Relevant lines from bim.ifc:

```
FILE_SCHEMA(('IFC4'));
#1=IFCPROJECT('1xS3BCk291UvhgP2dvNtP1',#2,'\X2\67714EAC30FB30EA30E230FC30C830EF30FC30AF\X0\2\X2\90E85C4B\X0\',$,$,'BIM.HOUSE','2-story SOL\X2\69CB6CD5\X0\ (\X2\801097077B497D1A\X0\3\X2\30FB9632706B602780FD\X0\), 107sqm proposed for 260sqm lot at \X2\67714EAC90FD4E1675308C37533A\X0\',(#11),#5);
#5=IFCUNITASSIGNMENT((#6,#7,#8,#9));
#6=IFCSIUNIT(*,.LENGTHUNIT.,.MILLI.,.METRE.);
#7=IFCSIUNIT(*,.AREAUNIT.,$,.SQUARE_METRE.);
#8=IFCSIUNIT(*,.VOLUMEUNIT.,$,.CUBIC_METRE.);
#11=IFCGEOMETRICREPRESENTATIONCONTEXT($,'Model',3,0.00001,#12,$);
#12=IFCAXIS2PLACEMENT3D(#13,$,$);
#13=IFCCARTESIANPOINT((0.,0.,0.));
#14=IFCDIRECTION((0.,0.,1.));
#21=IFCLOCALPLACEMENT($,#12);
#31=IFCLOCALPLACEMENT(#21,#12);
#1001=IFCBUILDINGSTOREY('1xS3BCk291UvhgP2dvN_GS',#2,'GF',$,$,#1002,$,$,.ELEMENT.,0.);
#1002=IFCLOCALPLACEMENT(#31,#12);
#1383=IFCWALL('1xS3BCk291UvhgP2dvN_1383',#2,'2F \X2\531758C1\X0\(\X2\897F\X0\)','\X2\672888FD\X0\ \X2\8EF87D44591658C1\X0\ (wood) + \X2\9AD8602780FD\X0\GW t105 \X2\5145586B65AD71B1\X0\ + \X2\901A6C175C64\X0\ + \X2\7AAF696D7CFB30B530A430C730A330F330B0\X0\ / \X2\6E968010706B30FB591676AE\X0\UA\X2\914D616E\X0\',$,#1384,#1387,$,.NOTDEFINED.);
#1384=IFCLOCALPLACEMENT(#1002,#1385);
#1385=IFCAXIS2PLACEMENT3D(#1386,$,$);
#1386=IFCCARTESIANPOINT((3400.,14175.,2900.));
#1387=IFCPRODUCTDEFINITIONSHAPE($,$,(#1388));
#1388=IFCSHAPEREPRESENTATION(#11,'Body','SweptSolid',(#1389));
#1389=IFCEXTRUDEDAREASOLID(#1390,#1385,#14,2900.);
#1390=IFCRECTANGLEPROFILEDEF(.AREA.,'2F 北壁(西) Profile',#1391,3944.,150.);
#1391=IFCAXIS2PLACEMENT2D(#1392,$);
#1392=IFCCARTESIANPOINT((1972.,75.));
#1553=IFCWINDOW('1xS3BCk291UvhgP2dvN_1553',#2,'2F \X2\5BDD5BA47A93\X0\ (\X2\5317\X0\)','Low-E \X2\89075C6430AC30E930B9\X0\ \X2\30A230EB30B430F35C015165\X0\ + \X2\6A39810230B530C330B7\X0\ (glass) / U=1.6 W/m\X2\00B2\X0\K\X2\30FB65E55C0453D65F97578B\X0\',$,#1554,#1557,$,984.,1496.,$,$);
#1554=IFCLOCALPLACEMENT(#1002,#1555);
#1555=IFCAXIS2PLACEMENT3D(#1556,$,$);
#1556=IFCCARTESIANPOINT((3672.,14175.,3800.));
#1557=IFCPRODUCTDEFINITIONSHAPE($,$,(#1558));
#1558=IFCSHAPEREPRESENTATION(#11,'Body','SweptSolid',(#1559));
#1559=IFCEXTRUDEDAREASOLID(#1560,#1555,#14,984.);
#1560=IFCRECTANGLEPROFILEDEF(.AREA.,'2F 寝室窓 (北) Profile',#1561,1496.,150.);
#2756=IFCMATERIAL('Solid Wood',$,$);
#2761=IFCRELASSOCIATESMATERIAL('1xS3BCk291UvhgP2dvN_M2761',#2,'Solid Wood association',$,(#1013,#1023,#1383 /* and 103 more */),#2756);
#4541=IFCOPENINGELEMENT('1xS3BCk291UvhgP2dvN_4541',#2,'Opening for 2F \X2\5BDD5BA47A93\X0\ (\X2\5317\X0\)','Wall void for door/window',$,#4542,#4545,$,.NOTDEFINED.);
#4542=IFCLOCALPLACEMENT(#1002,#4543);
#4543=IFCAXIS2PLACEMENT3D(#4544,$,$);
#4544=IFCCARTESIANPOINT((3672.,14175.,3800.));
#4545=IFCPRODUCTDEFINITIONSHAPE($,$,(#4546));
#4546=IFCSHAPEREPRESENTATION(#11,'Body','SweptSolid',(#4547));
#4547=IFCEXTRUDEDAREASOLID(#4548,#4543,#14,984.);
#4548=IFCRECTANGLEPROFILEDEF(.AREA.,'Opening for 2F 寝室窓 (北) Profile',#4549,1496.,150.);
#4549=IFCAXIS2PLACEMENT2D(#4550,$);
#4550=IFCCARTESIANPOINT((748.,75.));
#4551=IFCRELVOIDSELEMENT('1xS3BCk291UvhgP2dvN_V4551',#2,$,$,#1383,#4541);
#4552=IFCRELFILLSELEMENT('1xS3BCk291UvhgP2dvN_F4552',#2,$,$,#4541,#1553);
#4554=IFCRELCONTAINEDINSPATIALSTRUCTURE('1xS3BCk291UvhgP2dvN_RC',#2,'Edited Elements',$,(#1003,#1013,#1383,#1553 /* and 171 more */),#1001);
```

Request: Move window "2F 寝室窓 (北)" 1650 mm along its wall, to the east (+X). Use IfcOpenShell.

```python
import ifcopenshell
import ifcopenshell.api.geometry
import ifcopenshell.util.placement
import ifcopenshell.util.unit

model = ifcopenshell.open("bim.ifc")
unit_scale = ifcopenshell.util.unit.calculate_unit_scale(model)

window = model.by_id(1553)
opening = window.FillsVoids[0].RelatingOpeningElement
wall = opening.VoidsElements[0].RelatingBuildingElement

wall_matrix = ifcopenshell.util.placement.get_local_placement(wall.ObjectPlacement)
shift = wall_matrix[:3, 0] * 1.65 / unit_scale
before = ifcopenshell.util.placement.get_local_placement(window.ObjectPlacement)[:3, 3].copy()

# The window is not placed relative to its opening, so move both.
for product in (opening, window):
    matrix = ifcopenshell.util.placement.get_local_placement(product.ObjectPlacement)
    matrix[:3, 3] += shift
    ifcopenshell.api.geometry.edit_object_placement(model, product=product, matrix=matrix, is_si=False)

after = ifcopenshell.util.placement.get_local_placement(window.ObjectPlacement)[:3, 3]
print("window moved by", (after - before).round(3) + 0.0)

model.write("bim_v2.ifc")
```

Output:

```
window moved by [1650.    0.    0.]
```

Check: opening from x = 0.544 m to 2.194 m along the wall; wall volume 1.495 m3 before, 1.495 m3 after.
